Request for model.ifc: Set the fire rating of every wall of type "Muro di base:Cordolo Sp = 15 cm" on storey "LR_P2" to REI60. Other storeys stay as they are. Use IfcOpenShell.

First a look at what the model holds.

```python
import ifcopenshell
import ifcopenshell.util.element

model = ifcopenshell.open("model.ifc")
print(model.schema)
storey = next(s for s in model.by_type("IfcBuildingStorey") if s.Name == "LR_P2")
walls = [e for e in ifcopenshell.util.element.get_decomposition(storey) if e.is_a("IfcWall")]
seen = {}
for e in walls:
    element_type = ifcopenshell.util.element.get_type(e)
    key = (element_type.Name if element_type != e and element_type else None, ifcopenshell.util.element.get_pset(e, "Pset_WallCommon", "FireRating"))
    seen[key] = seen.get(key, 0) + 1
for (name, value), count in sorted(seen.items(), key=str):
    print(count, "x", name, "|", value)
```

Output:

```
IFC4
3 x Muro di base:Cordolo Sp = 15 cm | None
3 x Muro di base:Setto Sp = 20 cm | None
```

```python
import ifcopenshell
import ifcopenshell.api.pset
import ifcopenshell.util.element

model = ifcopenshell.open("model.ifc")

storey = next(s for s in model.by_type("IfcBuildingStorey") if s.Name == "LR_P2")
walls = [e for e in ifcopenshell.util.element.get_decomposition(storey) if e.is_a("IfcWall")]

count = 0
for e in walls:
    element_type = ifcopenshell.util.element.get_type(e)
    if element_type in (None, e) or element_type.Name != "Muro di base:Cordolo Sp = 15 cm":
        continue
    # add_pset returns the element's existing set when there is one.
    pset = ifcopenshell.api.pset.add_pset(model, product=e, name="Pset_WallCommon")
    ifcopenshell.api.pset.edit_pset(model, pset=pset, properties={"FireRating": "REI60"})
    count += 1

print(count, "walls updated")

model.write("model_v2.ifc")
```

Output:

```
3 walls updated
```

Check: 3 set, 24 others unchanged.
